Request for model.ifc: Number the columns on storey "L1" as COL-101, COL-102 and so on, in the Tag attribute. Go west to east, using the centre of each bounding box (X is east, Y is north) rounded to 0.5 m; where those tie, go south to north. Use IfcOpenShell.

First a look at what the model holds.

```python
import ifcopenshell
import ifcopenshell.util.element
import ifcopenshell.util.placement

model = ifcopenshell.open("model.ifc")
print(model.schema)
storey = next(s for s in model.by_type("IfcBuildingStorey") if s.Name == "L1")
columns = [e for e in ifcopenshell.util.element.get_decomposition(storey) if e.is_a("IfcColumn")]
for e in sorted(columns, key=lambda e: e.id()):
    origin = ifcopenshell.util.placement.get_local_placement(e.ObjectPlacement)[:3, 3]
    print(e.id(), e.Tag, e.Name, origin.round(2) + 0.0, sep=" | ")
```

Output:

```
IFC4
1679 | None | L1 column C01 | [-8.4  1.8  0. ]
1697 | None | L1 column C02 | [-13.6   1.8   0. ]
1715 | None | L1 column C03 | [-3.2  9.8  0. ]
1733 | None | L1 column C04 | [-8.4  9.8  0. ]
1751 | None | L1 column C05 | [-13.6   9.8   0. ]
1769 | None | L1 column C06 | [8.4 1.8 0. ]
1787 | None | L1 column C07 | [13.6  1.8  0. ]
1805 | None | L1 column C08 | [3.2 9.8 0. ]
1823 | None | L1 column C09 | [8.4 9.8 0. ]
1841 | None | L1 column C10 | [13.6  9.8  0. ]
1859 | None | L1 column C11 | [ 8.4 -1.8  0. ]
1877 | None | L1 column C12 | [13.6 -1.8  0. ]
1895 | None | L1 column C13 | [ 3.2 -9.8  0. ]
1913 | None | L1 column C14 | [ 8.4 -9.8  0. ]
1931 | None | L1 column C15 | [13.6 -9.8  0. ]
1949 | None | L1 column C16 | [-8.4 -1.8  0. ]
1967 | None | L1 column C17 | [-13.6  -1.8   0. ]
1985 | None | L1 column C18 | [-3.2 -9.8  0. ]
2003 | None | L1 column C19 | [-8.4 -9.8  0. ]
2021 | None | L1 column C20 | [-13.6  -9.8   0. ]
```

```python
import ifcopenshell
import ifcopenshell.geom
import ifcopenshell.util.element
import ifcopenshell.util.shape

model = ifcopenshell.open("model.ifc")
settings = ifcopenshell.geom.settings()
settings.set("use-world-coords", True)


def centre(element):
    shape = ifcopenshell.geom.create_shape(settings, element)
    return ifcopenshell.util.shape.get_bbox_centroid(shape.geometry)


storey = next(s for s in model.by_type("IfcBuildingStorey") if s.Name == "L1")
columns = [e for e in ifcopenshell.util.element.get_decomposition(storey) if e.is_a("IfcColumn")]

# Insertion points can sit at a corner or the storey origin, so sort by the geometry (in metres).
centres = {e: centre(e) for e in columns}
columns.sort(key=lambda e: (round(centres[e][0] / 0.5), centres[e][1]))

for i, e in enumerate(columns, start=1):
    number = f"COL-1{i:02d}"
    e.Tag = number
    print(e.id(), number)

model.write("model_edited.ifc")
```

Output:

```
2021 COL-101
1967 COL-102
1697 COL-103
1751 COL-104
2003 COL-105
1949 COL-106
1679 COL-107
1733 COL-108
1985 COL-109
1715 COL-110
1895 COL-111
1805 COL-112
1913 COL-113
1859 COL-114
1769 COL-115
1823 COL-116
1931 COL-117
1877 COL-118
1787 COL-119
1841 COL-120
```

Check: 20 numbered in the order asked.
